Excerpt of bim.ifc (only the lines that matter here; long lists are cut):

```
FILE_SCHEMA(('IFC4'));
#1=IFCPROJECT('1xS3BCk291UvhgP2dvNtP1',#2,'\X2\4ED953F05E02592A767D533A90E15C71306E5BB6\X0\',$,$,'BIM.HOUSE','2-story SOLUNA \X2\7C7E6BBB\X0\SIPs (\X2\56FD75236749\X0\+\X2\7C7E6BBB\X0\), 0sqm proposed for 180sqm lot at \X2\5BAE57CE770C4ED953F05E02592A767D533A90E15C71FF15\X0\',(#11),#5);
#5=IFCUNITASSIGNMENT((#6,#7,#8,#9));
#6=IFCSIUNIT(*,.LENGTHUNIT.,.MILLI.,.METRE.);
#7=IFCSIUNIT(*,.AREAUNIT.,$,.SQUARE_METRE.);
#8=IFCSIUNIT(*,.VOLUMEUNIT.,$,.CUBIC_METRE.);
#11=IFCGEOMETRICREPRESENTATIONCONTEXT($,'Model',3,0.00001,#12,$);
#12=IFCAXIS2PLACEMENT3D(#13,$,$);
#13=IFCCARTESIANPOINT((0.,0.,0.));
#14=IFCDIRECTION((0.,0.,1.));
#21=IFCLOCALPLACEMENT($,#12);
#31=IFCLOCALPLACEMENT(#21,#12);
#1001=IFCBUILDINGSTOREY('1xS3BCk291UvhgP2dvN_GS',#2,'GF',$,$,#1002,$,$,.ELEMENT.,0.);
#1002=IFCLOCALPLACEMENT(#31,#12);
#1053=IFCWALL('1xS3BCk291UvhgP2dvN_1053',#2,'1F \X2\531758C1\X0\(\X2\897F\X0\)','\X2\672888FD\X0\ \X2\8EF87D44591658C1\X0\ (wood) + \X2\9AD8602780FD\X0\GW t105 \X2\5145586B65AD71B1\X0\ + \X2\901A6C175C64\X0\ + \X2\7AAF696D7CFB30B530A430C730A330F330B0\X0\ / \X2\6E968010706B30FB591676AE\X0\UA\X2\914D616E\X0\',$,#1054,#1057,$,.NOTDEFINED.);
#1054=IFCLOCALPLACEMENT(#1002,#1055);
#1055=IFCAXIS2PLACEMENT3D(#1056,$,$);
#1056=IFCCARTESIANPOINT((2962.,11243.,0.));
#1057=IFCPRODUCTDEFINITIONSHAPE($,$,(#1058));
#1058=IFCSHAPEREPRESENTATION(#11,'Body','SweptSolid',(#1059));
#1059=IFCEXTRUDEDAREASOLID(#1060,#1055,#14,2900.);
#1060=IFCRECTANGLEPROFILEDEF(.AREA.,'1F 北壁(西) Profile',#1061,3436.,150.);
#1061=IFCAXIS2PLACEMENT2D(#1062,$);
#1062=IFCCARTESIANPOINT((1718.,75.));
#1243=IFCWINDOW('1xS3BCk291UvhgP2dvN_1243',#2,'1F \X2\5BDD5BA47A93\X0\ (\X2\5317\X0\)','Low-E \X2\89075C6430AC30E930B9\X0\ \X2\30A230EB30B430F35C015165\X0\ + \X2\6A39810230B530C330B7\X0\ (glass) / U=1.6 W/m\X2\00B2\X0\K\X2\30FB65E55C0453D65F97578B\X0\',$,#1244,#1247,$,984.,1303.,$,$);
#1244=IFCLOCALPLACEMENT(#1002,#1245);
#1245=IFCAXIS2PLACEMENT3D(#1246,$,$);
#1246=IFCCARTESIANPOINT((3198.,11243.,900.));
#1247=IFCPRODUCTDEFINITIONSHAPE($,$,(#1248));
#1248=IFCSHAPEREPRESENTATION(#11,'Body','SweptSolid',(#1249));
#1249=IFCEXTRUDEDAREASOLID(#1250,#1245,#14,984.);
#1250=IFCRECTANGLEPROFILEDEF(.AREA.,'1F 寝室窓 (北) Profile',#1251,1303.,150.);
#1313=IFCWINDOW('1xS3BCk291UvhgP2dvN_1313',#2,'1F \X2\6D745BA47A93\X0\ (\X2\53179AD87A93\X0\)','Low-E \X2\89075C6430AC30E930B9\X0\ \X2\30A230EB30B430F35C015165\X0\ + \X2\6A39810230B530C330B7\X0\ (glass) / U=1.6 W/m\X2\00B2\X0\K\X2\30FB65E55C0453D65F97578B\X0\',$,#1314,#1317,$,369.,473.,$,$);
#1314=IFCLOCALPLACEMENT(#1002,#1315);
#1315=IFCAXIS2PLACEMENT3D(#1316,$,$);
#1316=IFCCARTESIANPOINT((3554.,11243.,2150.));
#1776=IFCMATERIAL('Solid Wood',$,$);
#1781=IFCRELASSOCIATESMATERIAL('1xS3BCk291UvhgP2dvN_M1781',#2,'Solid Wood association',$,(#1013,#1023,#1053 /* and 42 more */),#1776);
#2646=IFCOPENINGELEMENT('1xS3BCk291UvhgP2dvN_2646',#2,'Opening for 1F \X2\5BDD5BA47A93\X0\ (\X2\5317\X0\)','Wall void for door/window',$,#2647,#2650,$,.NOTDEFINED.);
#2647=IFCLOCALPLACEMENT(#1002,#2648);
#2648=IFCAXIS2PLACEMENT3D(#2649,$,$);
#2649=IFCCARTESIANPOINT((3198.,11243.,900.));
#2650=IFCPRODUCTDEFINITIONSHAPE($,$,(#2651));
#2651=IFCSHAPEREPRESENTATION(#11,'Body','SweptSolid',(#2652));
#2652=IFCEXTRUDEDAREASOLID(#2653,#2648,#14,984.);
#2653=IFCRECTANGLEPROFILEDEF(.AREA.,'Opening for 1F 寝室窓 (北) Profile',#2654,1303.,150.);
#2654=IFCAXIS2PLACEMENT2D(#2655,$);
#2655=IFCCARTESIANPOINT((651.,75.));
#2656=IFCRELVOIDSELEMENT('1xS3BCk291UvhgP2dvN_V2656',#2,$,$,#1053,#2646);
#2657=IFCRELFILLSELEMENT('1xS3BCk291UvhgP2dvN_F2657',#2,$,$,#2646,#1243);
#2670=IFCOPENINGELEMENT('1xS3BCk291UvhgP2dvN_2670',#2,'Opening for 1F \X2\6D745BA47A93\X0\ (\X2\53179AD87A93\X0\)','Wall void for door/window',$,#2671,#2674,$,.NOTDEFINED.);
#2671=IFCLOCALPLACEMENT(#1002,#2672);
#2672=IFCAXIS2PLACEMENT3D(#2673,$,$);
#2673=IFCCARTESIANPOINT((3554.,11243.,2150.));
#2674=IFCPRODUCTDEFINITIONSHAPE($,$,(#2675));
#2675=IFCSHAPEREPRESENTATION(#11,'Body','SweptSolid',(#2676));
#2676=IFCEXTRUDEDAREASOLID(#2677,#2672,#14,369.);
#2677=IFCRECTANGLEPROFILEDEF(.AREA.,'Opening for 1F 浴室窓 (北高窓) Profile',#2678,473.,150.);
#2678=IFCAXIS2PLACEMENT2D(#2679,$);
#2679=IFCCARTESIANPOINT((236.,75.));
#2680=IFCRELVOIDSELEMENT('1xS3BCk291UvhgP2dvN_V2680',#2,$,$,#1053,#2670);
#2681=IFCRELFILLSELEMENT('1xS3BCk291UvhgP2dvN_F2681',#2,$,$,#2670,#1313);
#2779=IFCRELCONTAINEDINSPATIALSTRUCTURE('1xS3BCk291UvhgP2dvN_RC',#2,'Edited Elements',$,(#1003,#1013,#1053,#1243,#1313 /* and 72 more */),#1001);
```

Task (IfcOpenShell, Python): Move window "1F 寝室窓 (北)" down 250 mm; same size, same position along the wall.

```python
import numpy as np
import ifcopenshell
import ifcopenshell.api.geometry
import ifcopenshell.util.placement
import ifcopenshell.util.unit

model = ifcopenshell.open("bim.ifc")
unit_scale = ifcopenshell.util.unit.calculate_unit_scale(model)

window = model.by_guid("1xS3BCk291UvhgP2dvN_1243")
opening = window.FillsVoids[0].RelatingOpeningElement
dz = -0.25 / unit_scale

shift = np.array([0.0, 0.0, dz])
# The window is not placed relative to its opening, so move both.
for product in (opening, window):
    matrix = ifcopenshell.util.placement.get_local_placement(product.ObjectPlacement)
    matrix[:3, 3] += shift
    ifcopenshell.api.geometry.edit_object_placement(model, product=product, matrix=matrix, is_si=False)

print(f"moved by {dz * unit_scale:+.3f} m")

model.write("bim_edited.ifc")
```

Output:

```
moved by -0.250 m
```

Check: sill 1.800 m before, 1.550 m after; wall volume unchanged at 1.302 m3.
